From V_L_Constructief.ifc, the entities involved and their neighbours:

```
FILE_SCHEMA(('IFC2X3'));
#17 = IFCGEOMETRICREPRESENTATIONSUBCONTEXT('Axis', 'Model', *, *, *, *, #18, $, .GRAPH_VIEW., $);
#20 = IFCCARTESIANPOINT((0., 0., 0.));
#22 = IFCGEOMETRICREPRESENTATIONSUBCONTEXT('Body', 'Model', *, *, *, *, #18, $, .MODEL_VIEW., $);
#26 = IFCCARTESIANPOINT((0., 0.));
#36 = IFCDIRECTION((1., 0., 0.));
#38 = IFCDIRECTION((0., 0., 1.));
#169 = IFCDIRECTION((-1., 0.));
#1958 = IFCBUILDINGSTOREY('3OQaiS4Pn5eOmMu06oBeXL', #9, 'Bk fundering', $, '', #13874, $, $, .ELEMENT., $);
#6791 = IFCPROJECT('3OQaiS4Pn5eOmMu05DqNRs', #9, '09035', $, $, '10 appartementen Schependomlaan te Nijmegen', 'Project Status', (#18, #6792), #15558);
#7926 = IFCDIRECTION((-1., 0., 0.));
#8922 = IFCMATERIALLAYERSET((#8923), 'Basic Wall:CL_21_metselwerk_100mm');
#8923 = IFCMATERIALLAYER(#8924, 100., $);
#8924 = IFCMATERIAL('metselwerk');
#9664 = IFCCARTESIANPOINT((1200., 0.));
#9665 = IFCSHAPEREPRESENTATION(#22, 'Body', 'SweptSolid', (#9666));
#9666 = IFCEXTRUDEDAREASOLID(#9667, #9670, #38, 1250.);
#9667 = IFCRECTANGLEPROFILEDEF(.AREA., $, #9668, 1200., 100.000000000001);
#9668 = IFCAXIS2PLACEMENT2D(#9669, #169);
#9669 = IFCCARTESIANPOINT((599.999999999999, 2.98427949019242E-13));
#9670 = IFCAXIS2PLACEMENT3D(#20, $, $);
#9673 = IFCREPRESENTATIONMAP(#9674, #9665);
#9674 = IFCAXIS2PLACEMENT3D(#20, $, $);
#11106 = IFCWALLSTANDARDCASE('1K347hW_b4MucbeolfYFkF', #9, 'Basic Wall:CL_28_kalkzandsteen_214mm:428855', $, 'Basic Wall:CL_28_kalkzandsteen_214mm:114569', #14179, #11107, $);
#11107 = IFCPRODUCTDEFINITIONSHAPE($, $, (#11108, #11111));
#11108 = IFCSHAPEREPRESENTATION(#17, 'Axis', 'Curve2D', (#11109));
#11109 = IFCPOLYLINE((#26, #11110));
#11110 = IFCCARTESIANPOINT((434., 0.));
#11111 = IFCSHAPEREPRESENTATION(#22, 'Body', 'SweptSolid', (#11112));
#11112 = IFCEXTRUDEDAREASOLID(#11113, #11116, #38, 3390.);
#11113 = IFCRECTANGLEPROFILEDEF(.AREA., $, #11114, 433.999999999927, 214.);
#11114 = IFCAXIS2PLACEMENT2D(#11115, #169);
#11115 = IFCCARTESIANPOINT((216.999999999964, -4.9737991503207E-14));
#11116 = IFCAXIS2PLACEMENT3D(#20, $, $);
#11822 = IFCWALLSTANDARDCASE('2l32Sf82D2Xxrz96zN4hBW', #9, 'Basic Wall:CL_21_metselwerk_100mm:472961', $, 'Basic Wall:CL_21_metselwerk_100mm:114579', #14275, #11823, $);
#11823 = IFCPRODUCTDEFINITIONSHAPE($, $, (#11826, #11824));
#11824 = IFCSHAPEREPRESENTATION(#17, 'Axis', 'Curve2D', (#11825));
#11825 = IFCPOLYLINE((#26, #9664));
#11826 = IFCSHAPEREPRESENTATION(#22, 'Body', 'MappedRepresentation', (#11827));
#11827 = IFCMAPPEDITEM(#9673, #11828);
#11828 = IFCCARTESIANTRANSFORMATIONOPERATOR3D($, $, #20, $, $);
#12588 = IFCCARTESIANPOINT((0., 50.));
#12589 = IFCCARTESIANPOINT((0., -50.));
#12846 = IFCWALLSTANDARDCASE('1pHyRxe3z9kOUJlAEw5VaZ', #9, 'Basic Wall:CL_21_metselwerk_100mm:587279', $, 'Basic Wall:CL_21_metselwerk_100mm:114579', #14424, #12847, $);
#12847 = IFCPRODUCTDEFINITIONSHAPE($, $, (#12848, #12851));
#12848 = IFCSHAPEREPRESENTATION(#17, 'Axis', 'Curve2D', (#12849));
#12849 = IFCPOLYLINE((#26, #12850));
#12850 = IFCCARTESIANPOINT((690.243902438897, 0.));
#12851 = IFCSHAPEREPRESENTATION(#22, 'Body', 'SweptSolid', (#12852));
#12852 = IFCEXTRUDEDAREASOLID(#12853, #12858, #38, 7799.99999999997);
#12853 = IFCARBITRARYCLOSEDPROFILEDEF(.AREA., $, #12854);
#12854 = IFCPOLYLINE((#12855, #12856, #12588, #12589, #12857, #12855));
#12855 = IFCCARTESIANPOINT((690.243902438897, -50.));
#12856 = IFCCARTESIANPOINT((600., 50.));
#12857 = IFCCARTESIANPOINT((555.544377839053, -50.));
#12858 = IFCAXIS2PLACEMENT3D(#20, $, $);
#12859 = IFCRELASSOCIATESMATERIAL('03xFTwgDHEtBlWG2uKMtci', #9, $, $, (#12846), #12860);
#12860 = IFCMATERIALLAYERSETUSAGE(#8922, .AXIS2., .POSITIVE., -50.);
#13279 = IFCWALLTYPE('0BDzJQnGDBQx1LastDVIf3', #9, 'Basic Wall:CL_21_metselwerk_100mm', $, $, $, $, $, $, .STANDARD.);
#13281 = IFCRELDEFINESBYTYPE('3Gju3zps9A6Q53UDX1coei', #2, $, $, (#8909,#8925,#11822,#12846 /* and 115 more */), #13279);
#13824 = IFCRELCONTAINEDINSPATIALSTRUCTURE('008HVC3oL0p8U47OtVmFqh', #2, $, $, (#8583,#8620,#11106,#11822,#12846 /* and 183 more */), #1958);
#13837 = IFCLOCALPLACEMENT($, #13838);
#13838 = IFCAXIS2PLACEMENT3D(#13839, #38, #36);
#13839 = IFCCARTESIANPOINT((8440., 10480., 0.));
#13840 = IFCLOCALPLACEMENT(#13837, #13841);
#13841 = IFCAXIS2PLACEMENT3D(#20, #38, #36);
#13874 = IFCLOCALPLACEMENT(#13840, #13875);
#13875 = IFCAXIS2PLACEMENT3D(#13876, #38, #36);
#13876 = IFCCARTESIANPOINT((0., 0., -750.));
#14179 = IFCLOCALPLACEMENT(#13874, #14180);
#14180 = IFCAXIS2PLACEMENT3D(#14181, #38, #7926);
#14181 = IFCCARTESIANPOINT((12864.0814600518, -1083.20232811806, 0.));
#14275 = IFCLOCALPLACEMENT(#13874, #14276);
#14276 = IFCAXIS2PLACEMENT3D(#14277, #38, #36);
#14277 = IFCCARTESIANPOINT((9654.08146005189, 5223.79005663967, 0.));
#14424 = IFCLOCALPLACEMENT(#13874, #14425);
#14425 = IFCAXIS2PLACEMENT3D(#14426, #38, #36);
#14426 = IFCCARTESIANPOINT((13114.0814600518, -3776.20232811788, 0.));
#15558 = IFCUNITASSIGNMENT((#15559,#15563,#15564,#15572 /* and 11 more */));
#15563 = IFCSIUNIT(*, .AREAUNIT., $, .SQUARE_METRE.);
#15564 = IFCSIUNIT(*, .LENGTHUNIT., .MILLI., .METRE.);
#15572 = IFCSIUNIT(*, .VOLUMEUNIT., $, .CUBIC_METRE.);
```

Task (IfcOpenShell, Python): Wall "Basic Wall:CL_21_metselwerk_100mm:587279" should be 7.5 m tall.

```python
import ifcopenshell
import ifcopenshell.geom
import ifcopenshell.util.representation
import ifcopenshell.util.shape

model = ifcopenshell.open("V_L_Constructief.ifc")
settings = ifcopenshell.geom.settings()


def volume(element):
    """Net volume in cubic metres, openings subtracted."""
    shape = ifcopenshell.geom.create_shape(settings, element)
    return ifcopenshell.util.shape.get_volume(shape.geometry)


wall = model.by_guid("1pHyRxe3z9kOUJlAEw5VaZ")
before = volume(wall)

body = ifcopenshell.util.representation.get_representation(wall, "Model", "Body")
solid = body.Items[0]
old_height = solid.Depth
solid.Depth = 7500.0
after = volume(wall)

print(f"height {old_height:g} -> {solid.Depth:g}, volume {before:.3f} -> {after:.3f} m3")

model.write("V_L_Constructief_updated.ifc")
```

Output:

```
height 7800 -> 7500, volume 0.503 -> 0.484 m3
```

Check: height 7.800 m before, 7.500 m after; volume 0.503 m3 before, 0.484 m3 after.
